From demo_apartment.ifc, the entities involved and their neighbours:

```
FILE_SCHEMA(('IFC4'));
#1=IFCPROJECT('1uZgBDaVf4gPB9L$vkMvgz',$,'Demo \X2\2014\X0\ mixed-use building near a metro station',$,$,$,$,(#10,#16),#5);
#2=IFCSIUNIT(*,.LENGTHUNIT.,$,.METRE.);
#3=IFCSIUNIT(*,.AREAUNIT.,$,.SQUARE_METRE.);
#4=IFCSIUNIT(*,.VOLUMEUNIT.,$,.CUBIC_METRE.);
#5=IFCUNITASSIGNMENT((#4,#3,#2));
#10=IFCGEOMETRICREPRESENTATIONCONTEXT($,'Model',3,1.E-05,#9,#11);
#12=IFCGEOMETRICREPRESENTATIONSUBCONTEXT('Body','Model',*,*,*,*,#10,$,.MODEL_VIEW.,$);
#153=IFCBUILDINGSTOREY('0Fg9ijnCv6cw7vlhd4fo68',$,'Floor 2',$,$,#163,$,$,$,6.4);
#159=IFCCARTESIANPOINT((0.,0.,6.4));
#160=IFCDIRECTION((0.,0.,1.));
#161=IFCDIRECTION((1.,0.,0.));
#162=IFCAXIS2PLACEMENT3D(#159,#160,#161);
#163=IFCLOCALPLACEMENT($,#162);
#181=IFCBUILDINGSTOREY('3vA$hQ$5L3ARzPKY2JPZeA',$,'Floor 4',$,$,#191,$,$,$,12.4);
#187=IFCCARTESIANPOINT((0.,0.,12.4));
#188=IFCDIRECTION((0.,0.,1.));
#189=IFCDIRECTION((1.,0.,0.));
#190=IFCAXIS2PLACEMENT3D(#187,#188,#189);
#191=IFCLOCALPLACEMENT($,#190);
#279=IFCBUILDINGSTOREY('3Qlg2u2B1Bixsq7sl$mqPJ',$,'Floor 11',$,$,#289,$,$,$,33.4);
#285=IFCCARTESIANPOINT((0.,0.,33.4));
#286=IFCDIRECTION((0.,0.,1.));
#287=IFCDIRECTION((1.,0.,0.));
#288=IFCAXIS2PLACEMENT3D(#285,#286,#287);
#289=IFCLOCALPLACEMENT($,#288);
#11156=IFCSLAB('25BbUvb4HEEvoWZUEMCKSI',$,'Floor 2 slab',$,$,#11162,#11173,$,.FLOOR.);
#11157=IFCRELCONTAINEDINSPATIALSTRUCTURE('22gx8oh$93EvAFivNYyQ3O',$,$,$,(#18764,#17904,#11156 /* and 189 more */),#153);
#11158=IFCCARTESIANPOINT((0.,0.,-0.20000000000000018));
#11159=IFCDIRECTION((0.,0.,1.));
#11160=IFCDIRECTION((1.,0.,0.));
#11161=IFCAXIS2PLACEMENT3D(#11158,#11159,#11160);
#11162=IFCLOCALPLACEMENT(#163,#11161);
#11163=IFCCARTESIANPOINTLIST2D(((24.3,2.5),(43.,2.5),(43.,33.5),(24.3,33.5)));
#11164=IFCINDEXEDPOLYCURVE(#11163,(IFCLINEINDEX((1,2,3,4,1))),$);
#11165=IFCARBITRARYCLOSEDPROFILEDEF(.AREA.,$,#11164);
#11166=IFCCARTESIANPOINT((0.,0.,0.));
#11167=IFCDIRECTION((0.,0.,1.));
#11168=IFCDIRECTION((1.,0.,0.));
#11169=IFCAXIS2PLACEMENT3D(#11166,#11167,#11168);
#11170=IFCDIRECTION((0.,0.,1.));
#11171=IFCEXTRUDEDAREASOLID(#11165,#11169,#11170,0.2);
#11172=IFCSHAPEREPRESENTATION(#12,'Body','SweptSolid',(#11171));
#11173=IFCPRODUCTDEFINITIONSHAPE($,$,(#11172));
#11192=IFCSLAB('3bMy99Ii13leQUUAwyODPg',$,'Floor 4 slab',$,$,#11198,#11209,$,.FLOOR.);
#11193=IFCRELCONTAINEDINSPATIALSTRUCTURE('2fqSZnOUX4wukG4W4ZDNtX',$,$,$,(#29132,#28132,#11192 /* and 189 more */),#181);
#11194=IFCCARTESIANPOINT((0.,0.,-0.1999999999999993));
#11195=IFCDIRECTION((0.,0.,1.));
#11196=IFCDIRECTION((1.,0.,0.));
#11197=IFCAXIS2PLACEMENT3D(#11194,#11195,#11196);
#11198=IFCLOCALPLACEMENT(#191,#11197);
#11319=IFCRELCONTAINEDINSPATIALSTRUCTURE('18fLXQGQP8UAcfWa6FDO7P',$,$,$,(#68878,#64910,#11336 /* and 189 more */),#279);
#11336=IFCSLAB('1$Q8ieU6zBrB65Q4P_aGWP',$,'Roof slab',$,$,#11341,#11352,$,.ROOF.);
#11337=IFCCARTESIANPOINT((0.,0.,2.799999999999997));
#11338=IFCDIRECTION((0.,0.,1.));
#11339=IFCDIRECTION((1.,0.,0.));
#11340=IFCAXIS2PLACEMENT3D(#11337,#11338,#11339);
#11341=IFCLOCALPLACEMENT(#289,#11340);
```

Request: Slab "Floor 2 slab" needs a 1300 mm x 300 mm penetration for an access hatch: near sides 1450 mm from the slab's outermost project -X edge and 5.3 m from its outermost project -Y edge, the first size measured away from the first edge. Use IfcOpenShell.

```python
import numpy as np
import ifcopenshell
import ifcopenshell.api.feature
import ifcopenshell.api.geometry
import ifcopenshell.api.root
import ifcopenshell.geom
import ifcopenshell.util.placement
import ifcopenshell.util.representation
import ifcopenshell.util.shape
import ifcopenshell.util.unit

model = ifcopenshell.open("demo_apartment.ifc")
unit_scale = ifcopenshell.util.unit.calculate_unit_scale(model)
settings = ifcopenshell.geom.settings()


def volume(element):
    """Net volume in cubic metres, openings subtracted."""
    shape = ifcopenshell.geom.create_shape(settings, element)
    return ifcopenshell.util.shape.get_volume(shape.geometry)


slab = model.by_guid("25BbUvb4HEEvoWZUEMCKSI")
before = volume(slab)

# Extent in the slab's own axes, in metres. The edges named are its -X and -Y sides.
slab_shape = ifcopenshell.geom.create_shape(settings, slab)
vertices = ifcopenshell.util.shape.get_vertices(slab_shape.geometry)
x_min, y_min, bottom = vertices.min(axis=0)
top = vertices[:, 2].max()

opening = ifcopenshell.api.root.create_entity(model, ifc_class="IfcOpeningElement", name="Access hatch opening", predefined_type="OPENING")
context = ifcopenshell.util.representation.get_context(model, "Model", "Body", "MODEL_VIEW")
width, depth = 1.3, 0.3
outline = [(0.0, 0.0), (width, 0.0), (width, depth), (0.0, depth), (0.0, 0.0)]
# Overshoot both faces by 50 mm so the cut is clean.
shape = ifcopenshell.api.geometry.add_slab_representation(
    model, context=context, depth=top - bottom + 0.1, polyline=outline
)
ifcopenshell.api.geometry.assign_representation(model, product=opening, representation=shape)

matrix = ifcopenshell.util.placement.get_local_placement(slab.ObjectPlacement)
matrix[:, 3] = matrix @ np.append(np.array([x_min + 1.45, y_min + 5.3, bottom - 0.05]) / unit_scale, 1.0)
ifcopenshell.api.geometry.edit_object_placement(model, product=opening, matrix=matrix, is_si=False)
ifcopenshell.api.feature.add_feature(model, feature=opening, element=slab)

after = volume(slab)

print(f"slab volume {before:.3f} -> {after:.3f} m3")

model.write("demo_apartment_edited.ifc")
```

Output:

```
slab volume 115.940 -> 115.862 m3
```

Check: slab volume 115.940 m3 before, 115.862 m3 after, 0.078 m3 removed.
